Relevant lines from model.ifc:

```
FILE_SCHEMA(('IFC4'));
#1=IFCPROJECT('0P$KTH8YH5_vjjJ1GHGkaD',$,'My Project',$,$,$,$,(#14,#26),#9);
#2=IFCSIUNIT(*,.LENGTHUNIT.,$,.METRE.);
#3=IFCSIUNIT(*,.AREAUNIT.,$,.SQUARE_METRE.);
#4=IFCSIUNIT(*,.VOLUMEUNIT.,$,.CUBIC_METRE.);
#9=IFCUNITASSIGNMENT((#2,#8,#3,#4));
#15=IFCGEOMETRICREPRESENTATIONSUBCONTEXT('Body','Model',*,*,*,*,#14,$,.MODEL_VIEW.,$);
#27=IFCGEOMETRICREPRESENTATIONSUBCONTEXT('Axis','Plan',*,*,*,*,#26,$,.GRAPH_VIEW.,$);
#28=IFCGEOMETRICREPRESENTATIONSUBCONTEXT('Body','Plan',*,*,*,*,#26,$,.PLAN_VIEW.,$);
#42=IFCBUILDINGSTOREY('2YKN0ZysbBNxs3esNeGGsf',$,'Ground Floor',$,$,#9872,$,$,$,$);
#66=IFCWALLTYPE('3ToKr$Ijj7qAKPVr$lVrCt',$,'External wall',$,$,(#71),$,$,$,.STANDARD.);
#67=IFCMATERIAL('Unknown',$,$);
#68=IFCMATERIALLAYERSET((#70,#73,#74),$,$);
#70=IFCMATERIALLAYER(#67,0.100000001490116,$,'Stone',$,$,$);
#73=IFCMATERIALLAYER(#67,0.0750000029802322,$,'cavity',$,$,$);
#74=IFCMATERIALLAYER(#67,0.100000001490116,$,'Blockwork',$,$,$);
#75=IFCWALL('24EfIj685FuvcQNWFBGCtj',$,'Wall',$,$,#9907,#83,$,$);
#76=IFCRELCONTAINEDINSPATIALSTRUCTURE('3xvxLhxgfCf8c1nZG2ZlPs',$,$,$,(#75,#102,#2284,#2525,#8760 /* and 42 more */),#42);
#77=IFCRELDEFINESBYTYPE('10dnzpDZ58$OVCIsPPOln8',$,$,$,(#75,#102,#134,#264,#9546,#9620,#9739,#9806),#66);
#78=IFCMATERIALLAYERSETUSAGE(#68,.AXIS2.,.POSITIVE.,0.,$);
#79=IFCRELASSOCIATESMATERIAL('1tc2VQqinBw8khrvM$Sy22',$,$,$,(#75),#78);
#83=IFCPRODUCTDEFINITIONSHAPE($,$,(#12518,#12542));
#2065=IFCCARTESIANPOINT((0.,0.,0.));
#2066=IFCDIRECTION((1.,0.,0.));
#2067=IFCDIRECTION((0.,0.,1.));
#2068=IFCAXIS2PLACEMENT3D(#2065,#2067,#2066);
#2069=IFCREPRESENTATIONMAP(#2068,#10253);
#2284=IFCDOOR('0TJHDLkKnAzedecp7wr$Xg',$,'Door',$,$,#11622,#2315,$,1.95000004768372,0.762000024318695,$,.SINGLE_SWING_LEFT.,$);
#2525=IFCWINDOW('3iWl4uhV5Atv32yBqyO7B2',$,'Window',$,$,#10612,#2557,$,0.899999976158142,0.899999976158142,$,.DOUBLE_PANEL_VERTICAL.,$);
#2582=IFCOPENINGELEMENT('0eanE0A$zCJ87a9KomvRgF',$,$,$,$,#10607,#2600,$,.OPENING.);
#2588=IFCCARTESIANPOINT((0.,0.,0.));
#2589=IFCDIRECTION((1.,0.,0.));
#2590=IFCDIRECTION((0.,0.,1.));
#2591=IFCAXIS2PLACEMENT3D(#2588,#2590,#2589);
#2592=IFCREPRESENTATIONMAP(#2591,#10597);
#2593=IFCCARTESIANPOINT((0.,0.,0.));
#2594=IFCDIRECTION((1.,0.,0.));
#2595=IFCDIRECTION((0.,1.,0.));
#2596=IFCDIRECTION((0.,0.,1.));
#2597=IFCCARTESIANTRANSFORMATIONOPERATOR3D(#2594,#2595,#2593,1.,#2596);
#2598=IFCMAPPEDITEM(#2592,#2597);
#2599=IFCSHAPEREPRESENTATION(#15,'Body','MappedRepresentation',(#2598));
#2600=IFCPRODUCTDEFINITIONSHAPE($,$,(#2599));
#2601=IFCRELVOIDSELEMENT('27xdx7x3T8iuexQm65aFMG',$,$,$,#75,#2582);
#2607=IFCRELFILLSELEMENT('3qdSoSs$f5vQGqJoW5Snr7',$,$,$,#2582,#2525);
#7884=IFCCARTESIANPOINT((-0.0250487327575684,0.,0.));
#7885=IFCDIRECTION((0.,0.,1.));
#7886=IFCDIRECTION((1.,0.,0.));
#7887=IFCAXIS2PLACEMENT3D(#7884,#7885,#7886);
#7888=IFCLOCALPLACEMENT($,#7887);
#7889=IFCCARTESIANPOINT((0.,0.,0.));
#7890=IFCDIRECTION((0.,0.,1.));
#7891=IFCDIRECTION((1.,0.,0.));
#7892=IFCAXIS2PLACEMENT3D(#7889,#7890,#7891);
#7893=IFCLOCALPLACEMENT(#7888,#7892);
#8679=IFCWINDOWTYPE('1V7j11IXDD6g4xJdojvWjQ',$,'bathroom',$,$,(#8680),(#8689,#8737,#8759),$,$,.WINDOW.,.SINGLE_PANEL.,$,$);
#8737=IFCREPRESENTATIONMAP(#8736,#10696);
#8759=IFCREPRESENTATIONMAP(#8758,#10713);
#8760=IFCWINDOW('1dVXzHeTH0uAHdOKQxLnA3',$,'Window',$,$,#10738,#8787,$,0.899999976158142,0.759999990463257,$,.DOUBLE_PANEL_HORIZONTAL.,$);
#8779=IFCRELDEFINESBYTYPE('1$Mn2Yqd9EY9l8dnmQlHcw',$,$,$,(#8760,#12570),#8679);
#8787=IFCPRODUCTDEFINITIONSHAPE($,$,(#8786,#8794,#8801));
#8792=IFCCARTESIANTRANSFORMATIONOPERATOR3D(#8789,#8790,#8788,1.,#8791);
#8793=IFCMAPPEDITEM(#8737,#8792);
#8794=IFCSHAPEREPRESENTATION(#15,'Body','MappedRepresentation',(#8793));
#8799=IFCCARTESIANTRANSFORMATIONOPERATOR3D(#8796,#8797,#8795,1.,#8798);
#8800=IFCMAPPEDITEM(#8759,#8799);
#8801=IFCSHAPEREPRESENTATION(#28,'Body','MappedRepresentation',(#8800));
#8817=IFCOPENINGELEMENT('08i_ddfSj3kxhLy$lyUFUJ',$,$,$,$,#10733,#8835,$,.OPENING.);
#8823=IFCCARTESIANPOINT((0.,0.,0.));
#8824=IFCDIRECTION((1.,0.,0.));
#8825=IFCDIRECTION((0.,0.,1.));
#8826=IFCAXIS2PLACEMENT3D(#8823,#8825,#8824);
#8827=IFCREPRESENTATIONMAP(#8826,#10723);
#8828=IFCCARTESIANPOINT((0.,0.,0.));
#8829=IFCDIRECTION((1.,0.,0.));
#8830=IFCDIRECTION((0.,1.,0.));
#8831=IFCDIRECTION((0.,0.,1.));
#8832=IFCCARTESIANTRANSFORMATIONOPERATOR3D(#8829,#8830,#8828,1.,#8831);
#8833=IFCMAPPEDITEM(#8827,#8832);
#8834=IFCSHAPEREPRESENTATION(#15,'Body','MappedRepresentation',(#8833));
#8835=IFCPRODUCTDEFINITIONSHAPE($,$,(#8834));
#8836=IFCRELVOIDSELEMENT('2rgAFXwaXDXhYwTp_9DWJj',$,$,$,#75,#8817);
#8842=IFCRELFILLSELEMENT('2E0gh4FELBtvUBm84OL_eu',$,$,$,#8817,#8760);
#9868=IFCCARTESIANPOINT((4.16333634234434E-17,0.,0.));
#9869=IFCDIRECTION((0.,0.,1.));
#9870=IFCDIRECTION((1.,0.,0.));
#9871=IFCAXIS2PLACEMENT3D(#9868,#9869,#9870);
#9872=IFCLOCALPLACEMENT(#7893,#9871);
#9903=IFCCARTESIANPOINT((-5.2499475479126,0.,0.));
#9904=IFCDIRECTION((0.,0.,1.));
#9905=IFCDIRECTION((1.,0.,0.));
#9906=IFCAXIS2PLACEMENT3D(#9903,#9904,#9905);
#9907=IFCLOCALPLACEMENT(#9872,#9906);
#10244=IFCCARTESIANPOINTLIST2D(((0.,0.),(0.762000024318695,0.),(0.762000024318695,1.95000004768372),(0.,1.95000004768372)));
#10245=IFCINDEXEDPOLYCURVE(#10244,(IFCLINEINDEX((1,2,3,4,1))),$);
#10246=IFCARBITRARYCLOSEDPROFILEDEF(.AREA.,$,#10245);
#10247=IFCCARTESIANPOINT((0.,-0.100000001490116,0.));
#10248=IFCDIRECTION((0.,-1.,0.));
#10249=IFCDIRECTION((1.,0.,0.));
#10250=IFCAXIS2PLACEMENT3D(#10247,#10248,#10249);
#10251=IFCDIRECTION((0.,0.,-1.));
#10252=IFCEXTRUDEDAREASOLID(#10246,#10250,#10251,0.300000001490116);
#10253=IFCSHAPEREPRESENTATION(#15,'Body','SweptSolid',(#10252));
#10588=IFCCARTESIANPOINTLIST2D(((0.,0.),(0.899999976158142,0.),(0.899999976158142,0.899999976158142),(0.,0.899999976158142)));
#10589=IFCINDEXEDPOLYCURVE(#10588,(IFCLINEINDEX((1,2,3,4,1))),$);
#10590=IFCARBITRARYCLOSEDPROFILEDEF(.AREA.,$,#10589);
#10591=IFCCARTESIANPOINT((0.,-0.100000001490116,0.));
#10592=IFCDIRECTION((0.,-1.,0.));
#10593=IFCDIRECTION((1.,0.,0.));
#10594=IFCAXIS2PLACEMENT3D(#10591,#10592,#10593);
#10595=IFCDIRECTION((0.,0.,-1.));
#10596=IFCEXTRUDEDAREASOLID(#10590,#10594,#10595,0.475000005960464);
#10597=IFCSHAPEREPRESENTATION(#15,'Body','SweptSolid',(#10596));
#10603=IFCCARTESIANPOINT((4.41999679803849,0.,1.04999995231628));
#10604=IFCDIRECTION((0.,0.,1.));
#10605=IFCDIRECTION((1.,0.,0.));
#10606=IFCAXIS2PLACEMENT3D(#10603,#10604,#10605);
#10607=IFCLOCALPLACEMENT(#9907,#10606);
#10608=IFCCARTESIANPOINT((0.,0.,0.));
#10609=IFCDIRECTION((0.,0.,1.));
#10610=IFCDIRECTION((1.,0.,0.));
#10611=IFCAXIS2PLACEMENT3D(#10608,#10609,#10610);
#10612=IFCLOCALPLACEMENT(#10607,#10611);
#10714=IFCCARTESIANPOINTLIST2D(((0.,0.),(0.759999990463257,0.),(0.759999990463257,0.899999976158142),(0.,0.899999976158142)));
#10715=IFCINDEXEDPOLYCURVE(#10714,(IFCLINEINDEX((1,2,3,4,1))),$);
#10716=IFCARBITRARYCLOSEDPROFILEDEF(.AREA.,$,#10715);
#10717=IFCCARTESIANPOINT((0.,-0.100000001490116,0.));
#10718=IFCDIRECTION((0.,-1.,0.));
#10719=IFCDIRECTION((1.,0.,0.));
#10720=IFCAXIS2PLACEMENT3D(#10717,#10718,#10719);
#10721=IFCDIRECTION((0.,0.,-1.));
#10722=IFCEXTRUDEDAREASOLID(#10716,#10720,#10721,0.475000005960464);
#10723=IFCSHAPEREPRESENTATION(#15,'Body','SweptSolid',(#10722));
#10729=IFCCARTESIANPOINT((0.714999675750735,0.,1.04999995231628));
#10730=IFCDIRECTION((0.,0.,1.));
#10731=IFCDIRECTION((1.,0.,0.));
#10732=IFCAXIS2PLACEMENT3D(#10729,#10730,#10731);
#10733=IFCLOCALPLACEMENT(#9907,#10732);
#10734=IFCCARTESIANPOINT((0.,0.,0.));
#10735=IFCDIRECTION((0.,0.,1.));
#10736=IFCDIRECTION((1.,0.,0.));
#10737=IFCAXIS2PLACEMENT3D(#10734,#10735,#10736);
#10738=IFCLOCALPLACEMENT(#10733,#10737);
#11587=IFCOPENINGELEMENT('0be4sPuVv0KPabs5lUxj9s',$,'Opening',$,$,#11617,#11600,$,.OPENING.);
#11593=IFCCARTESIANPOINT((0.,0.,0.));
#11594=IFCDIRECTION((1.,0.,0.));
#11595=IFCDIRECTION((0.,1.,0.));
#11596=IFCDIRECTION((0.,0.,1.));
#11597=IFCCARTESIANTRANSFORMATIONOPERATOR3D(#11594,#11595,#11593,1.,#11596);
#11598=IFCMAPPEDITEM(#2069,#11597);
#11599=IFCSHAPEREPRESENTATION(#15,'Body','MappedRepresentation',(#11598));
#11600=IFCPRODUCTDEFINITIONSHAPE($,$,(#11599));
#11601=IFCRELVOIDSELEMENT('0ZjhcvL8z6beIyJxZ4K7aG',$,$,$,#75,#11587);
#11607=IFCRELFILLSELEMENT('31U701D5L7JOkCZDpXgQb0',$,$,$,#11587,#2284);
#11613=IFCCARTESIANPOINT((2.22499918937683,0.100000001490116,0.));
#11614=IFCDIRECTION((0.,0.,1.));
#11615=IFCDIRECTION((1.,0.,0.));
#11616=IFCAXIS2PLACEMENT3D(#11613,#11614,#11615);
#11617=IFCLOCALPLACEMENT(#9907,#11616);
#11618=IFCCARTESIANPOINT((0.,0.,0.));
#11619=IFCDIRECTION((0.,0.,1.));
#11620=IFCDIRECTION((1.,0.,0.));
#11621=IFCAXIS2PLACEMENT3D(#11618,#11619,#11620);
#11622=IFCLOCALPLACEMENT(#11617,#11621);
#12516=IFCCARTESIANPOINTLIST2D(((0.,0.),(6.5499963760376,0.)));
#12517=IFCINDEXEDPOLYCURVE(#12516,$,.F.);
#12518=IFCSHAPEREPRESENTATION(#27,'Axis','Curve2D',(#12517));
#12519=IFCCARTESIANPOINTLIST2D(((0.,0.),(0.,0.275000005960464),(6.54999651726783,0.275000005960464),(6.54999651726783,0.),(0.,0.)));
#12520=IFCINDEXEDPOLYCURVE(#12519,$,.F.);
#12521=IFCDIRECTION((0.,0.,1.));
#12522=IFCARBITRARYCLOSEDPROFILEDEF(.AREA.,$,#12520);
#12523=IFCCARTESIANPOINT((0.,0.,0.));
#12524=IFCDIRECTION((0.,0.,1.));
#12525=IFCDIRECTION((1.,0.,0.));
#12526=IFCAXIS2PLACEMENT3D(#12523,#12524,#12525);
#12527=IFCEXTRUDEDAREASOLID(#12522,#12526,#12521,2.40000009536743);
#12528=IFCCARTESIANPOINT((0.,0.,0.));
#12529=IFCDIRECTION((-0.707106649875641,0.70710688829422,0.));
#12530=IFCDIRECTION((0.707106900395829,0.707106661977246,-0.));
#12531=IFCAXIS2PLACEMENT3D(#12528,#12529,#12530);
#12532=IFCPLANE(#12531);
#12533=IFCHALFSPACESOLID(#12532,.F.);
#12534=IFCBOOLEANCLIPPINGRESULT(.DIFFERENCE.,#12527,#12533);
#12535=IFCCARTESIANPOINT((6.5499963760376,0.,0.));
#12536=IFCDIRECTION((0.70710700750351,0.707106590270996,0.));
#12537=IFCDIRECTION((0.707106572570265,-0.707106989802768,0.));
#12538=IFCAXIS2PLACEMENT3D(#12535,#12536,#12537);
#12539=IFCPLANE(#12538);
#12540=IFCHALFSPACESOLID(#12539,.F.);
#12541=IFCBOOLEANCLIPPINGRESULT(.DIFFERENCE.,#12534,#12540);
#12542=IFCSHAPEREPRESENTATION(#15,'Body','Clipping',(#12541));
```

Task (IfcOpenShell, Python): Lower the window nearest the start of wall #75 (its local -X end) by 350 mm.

```python
import numpy as np
import ifcopenshell
import ifcopenshell.api.geometry
import ifcopenshell.util.placement
import ifcopenshell.util.unit

model = ifcopenshell.open("model.ifc")
unit_scale = ifcopenshell.util.unit.calculate_unit_scale(model)

window = model.by_guid("1dVXzHeTH0uAHdOKQxLnA3")
opening = window.FillsVoids[0].RelatingOpeningElement
dz = -0.35 / unit_scale

shift = np.array([0.0, 0.0, dz])
# The window is placed relative to its opening, so it follows when the opening moves.
matrix = ifcopenshell.util.placement.get_local_placement(opening.ObjectPlacement)
matrix[:3, 3] += shift
ifcopenshell.api.geometry.edit_object_placement(
    model, product=opening, matrix=matrix, is_si=False, should_transform_children=True
)

print(f"moved by {dz * unit_scale:+.3f} m")

model.write("model_rev.ifc")
```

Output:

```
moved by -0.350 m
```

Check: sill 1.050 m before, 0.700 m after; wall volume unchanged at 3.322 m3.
